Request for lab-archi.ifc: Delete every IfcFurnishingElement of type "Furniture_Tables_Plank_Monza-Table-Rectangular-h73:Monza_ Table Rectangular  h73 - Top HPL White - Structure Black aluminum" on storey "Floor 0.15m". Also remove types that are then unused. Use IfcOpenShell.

First a look at what the model holds.

```python
import ifcopenshell
import ifcopenshell.util.element

model = ifcopenshell.open("lab-archi.ifc")
print(model.schema)
storey = next(s for s in model.by_type("IfcBuildingStorey") if s.Name == "Floor 0.15m")
furniture = [e for e in ifcopenshell.util.element.get_decomposition(storey) if e.is_a("IfcFurnishingElement")]
seen = {}
for e in furniture:
    element_type = ifcopenshell.util.element.get_type(e)
    name = element_type.Name if element_type not in (None, e) else None
    seen[name] = seen.get(name, 0) + 1
for name, count in sorted(seen.items(), key=str):
    print(count, "x", name)
```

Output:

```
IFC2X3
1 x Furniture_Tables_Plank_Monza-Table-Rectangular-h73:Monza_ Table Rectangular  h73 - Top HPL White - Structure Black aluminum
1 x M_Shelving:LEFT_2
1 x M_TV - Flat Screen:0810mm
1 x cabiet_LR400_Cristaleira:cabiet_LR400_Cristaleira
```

```python
import ifcopenshell
import ifcopenshell.api.root
import ifcopenshell.util.element

model = ifcopenshell.open("lab-archi.ifc")

storey = next(s for s in model.by_type("IfcBuildingStorey") if s.Name == "Floor 0.15m")
furniture = [e for e in ifcopenshell.util.element.get_decomposition(storey) if e.is_a("IfcFurnishingElement")]
targets = [e for e in furniture if (t := ifcopenshell.util.element.get_type(e)) not in (None, e) and t.Name == "Furniture_Tables_Plank_Monza-Table-Rectangular-h73:Monza_ Table Rectangular  h73 - Top HPL White - Structure Black aluminum"]
types = {ifcopenshell.util.element.get_type(e) for e in targets} - {None, *targets}

for e in targets:
    ifcopenshell.api.root.remove_product(model, product=e)
print(len(targets), "removed")

unused = [t for t in types if not ifcopenshell.util.element.get_types(t)]
for t in unused:
    ifcopenshell.api.root.remove_product(model, product=t)
print(len(unused), "unused types removed")

model.write("lab-archi_updated.ifc")
```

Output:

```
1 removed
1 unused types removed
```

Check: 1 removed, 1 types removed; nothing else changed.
